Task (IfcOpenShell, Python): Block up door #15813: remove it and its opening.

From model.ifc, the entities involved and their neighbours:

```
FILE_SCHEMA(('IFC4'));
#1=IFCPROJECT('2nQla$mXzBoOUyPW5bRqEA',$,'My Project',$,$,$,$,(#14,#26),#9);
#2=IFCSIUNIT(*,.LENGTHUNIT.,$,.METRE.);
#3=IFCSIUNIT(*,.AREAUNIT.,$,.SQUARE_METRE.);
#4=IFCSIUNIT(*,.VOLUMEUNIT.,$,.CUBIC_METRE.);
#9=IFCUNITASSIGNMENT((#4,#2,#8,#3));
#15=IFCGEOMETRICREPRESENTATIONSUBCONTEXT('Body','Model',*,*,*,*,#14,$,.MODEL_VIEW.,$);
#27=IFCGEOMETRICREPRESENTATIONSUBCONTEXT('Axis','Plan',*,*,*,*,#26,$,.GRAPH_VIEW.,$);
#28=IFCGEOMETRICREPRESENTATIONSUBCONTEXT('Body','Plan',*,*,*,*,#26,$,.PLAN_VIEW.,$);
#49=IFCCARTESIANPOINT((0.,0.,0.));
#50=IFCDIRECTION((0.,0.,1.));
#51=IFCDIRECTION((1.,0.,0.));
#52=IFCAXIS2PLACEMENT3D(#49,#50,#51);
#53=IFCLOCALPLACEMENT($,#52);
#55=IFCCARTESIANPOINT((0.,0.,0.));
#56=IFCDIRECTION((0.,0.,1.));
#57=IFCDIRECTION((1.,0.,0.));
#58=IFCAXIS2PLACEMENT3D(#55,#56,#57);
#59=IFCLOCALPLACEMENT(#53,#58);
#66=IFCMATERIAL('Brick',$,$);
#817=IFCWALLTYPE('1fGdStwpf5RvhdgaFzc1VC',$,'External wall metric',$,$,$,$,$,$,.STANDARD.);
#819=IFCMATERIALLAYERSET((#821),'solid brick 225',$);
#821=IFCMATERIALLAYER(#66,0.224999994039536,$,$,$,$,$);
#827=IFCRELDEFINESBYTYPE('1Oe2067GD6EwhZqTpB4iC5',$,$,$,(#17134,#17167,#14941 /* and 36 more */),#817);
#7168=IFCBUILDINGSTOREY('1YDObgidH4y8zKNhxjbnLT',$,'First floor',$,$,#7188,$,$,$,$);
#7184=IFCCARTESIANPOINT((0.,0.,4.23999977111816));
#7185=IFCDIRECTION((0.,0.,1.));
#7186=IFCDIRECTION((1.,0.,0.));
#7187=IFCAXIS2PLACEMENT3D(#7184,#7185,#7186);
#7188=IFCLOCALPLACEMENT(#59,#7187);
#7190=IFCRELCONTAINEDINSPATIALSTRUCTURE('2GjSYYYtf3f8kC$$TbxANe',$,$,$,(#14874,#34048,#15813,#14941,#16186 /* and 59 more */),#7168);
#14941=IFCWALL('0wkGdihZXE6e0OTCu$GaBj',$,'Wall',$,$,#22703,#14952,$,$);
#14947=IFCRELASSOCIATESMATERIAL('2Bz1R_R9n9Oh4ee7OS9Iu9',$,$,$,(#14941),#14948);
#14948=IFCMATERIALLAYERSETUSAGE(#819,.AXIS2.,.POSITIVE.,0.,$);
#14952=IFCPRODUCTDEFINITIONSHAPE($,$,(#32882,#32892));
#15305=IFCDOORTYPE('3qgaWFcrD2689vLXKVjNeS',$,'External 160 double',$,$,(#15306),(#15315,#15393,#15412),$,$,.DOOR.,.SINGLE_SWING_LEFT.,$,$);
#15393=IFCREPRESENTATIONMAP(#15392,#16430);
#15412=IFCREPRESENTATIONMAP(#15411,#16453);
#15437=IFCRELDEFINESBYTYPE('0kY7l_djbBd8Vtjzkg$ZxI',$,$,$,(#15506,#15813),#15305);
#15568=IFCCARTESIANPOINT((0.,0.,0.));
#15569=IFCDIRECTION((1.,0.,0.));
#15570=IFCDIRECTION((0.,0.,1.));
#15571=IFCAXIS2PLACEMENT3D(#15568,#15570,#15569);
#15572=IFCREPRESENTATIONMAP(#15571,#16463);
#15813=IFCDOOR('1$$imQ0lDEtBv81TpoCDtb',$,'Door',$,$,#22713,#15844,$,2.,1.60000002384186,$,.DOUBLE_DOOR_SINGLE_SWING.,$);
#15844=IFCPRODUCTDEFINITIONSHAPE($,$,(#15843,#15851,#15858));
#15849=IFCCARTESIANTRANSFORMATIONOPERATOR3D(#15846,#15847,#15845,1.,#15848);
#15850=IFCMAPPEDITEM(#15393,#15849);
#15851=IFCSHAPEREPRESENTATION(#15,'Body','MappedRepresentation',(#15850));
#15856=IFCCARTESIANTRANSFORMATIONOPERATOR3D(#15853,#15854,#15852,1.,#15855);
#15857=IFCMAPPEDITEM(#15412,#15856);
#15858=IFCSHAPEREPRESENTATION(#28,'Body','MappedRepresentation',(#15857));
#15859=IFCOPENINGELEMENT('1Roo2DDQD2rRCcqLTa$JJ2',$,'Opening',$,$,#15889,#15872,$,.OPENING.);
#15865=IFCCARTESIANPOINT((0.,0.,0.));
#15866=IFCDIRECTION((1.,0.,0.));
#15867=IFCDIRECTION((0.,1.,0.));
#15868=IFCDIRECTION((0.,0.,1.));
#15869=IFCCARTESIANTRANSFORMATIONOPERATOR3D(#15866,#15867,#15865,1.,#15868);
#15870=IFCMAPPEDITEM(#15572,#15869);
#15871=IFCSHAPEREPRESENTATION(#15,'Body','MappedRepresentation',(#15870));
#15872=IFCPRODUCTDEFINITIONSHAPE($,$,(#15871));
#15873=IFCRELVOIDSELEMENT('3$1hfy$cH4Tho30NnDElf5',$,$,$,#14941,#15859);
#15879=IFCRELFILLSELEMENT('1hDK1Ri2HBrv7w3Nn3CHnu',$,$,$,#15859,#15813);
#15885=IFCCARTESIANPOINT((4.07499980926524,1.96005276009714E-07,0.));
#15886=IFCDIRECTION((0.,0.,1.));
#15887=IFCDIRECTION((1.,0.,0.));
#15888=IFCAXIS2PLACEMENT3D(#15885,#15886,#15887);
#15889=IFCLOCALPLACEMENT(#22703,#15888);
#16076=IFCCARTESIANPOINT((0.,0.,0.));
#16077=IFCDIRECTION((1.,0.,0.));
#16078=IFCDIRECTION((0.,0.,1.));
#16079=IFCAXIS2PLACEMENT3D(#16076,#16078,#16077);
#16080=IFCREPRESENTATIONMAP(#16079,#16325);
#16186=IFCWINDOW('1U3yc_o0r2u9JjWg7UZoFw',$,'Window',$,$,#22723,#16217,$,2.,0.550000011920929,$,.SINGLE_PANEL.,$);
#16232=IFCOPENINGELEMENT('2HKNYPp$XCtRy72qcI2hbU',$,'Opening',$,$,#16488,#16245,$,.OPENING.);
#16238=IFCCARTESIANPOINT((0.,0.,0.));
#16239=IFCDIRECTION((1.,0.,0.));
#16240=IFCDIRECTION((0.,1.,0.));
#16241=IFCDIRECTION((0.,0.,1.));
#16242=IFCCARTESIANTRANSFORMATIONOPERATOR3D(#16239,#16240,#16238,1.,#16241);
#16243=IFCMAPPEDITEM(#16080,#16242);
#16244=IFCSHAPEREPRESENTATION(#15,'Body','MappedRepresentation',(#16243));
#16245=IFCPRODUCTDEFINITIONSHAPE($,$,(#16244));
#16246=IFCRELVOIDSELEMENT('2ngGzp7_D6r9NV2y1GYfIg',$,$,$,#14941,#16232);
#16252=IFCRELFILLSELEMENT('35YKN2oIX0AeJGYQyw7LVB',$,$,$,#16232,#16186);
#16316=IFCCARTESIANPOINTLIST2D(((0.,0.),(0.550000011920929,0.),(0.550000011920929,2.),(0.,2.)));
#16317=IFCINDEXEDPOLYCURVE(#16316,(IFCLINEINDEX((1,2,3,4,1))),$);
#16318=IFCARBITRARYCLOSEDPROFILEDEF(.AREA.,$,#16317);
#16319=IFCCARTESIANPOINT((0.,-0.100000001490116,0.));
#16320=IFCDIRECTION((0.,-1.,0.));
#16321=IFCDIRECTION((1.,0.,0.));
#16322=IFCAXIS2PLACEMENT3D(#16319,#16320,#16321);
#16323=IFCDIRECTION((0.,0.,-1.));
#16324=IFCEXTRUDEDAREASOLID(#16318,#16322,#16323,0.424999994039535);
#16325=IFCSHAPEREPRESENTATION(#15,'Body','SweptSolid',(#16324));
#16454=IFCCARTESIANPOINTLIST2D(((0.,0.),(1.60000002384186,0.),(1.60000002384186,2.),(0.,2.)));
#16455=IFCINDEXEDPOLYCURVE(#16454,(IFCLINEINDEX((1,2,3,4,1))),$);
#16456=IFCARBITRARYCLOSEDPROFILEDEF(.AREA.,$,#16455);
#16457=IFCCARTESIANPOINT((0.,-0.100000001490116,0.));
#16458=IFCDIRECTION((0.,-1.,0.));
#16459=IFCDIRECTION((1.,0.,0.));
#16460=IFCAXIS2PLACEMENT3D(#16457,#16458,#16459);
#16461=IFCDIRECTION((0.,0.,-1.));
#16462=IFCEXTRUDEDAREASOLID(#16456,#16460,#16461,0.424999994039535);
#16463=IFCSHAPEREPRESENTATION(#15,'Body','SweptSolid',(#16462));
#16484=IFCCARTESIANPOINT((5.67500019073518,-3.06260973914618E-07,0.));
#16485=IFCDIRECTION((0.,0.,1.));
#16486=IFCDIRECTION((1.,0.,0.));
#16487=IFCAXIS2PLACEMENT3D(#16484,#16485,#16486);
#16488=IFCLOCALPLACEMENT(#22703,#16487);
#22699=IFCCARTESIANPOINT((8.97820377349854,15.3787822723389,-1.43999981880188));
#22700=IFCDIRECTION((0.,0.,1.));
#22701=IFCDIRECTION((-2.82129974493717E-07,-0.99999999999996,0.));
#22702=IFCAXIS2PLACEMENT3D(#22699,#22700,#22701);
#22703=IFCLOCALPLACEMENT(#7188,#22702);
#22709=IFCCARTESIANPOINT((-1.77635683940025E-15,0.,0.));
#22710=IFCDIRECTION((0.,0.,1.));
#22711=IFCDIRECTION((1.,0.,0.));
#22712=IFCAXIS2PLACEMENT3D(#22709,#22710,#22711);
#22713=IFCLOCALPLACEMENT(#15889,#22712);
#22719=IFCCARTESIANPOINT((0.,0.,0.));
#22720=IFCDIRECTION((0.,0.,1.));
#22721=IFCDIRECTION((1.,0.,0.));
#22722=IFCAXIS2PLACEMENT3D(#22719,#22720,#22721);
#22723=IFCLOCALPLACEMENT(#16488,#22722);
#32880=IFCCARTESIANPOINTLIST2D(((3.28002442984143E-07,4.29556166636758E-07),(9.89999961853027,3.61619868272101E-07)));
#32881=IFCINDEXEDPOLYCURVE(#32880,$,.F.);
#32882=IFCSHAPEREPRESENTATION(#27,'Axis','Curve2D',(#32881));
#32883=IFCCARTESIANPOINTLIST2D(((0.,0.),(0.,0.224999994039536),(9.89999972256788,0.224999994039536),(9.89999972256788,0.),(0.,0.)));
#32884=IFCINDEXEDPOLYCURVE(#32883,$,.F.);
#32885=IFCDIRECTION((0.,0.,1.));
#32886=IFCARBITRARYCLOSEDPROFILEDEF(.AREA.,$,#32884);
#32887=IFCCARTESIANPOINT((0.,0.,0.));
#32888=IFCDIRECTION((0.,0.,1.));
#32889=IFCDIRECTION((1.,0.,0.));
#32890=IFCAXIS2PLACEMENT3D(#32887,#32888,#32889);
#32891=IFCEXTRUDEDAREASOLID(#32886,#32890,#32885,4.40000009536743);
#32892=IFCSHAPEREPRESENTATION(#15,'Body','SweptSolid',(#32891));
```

```python
import ifcopenshell
import ifcopenshell.api.feature
import ifcopenshell.api.root
import ifcopenshell.geom
import ifcopenshell.util.shape

model = ifcopenshell.open("model.ifc")
settings = ifcopenshell.geom.settings()


def volume(element):
    """Net volume in cubic metres, openings subtracted."""
    shape = ifcopenshell.geom.create_shape(settings, element)
    return ifcopenshell.util.shape.get_volume(shape.geometry)


door = model.by_guid("1$$imQ0lDEtBv81TpoCDtb")
opening = door.FillsVoids[0].RelatingOpeningElement
wall = opening.VoidsElements[0].RelatingBuildingElement
before = volume(wall)

ifcopenshell.api.root.remove_product(model, product=door)
ifcopenshell.api.feature.remove_feature(model, feature=opening)

after = volume(wall)

print(f"wall volume {before:.3f} -> {after:.3f} m3")

model.write("model-out.ifc")
```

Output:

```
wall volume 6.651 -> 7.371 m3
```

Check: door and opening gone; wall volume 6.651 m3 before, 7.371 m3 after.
